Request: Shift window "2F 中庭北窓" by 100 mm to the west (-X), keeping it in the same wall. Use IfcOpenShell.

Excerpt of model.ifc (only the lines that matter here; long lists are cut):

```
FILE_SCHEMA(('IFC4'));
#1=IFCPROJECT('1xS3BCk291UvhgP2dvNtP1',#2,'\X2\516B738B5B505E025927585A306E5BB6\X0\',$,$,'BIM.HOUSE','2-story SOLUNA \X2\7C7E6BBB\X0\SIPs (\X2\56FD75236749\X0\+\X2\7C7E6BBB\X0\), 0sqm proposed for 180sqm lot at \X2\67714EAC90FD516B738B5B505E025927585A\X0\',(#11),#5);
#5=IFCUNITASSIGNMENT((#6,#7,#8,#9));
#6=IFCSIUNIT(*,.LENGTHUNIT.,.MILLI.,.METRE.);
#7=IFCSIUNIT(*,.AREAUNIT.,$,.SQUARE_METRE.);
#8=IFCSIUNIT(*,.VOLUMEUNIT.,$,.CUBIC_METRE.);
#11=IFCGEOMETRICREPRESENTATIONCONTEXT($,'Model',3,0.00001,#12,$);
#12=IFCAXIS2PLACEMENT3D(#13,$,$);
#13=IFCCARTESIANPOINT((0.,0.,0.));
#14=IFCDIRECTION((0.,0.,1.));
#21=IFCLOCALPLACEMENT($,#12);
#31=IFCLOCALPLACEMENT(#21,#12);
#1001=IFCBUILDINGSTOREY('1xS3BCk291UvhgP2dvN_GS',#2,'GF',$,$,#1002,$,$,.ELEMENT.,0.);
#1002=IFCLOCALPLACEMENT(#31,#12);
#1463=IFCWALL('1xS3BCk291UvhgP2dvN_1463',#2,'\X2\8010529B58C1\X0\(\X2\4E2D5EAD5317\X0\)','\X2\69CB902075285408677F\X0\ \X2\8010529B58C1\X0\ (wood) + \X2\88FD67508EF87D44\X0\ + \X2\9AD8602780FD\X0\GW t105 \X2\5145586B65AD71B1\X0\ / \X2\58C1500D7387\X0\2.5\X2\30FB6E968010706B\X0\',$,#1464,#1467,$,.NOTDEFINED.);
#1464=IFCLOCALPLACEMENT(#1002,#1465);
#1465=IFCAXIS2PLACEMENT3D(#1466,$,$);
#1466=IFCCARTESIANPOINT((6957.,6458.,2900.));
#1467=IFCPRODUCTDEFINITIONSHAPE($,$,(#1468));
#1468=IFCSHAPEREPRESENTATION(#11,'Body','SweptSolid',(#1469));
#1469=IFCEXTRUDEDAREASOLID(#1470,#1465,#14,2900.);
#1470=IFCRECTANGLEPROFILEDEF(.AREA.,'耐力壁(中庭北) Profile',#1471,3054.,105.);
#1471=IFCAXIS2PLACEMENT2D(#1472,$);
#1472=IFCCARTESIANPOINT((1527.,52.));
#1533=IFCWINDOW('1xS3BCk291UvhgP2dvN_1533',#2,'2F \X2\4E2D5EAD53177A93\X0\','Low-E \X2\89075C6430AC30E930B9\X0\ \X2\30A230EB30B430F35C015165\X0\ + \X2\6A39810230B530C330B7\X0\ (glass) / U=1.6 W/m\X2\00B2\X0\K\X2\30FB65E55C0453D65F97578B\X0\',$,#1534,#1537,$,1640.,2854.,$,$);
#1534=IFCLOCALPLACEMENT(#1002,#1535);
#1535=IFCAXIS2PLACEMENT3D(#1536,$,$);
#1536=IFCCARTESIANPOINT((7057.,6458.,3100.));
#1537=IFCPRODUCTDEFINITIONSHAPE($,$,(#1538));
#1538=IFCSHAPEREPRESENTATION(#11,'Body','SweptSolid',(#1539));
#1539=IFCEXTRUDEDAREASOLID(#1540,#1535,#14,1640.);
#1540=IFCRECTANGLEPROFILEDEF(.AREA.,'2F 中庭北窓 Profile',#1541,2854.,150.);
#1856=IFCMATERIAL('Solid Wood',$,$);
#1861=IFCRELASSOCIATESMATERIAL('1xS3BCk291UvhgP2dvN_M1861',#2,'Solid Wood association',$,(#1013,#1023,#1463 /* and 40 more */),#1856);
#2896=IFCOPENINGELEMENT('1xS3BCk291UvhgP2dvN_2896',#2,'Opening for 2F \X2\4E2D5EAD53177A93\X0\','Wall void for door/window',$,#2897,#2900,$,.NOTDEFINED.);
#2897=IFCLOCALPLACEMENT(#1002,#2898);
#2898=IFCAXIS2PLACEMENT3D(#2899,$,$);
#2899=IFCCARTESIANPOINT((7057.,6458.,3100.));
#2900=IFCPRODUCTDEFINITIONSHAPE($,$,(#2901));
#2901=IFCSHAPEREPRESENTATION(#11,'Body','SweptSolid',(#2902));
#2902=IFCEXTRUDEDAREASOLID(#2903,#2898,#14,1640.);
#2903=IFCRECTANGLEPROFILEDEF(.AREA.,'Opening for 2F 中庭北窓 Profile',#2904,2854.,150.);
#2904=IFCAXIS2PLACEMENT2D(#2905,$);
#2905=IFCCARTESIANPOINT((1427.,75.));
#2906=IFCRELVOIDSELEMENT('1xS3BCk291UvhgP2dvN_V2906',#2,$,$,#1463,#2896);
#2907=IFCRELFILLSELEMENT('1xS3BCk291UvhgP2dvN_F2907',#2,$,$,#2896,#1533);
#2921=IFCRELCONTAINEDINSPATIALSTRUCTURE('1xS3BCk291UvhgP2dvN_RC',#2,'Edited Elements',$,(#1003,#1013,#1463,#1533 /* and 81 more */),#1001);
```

```python
import ifcopenshell
import ifcopenshell.api.geometry
import ifcopenshell.util.placement
import ifcopenshell.util.unit

model = ifcopenshell.open("model.ifc")
unit_scale = ifcopenshell.util.unit.calculate_unit_scale(model)

window = model.by_guid("1xS3BCk291UvhgP2dvN_1533")
opening = window.FillsVoids[0].RelatingOpeningElement
wall = opening.VoidsElements[0].RelatingBuildingElement

wall_matrix = ifcopenshell.util.placement.get_local_placement(wall.ObjectPlacement)
shift = wall_matrix[:3, 0] * -0.1 / unit_scale
before = ifcopenshell.util.placement.get_local_placement(window.ObjectPlacement)[:3, 3].copy()

# The window is not placed relative to its opening, so move both.
for product in (opening, window):
    matrix = ifcopenshell.util.placement.get_local_placement(product.ObjectPlacement)
    matrix[:3, 3] += shift
    ifcopenshell.api.geometry.edit_object_placement(model, product=product, matrix=matrix, is_si=False)

after = ifcopenshell.util.placement.get_local_placement(window.ObjectPlacement)[:3, 3]
print("window moved by", (after - before).round(3) + 0.0)

model.write("model_updated.ifc")
```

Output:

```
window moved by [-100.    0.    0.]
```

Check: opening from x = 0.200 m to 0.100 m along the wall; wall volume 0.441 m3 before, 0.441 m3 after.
